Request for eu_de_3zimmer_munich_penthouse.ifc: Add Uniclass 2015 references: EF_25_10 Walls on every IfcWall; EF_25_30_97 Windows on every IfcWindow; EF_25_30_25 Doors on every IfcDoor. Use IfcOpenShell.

First a look at what the model holds.

```python
import ifcopenshell

model = ifcopenshell.open("eu_de_3zimmer_munich_penthouse.ifc")
print(model.schema)
print("classifications:", [c.Name for c in model.by_type("IfcClassification")])
for ifc_class in ("IfcDoor", "IfcRoof", "IfcStair", "IfcWall", "IfcWindow"):
    print(ifc_class, len(model.by_type(ifc_class)))
```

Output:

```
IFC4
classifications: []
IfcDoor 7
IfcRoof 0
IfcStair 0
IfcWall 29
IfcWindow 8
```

```python
import ifcopenshell
import ifcopenshell.api.classification

model = ifcopenshell.open("eu_de_3zimmer_munich_penthouse.ifc")

system = ifcopenshell.api.classification.add_classification(model, classification="Uniclass 2015")

codes = {
    "IfcWall": ("EF_25_10", "Walls"),
    "IfcWindow": ("EF_25_30_97", "Windows"),
    "IfcDoor": ("EF_25_30_25", "Doors"),
}
for ifc_class, (code, name) in codes.items():
    products = model.by_type(ifc_class)
    ifcopenshell.api.classification.add_reference(
        model, products=products, classification=system, identification=code, name=name
    )
    print(code, len(products))

model.write("eu_de_3zimmer_munich_penthouse_edited.ifc")
```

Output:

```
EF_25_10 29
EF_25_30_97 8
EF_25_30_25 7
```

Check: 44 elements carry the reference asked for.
